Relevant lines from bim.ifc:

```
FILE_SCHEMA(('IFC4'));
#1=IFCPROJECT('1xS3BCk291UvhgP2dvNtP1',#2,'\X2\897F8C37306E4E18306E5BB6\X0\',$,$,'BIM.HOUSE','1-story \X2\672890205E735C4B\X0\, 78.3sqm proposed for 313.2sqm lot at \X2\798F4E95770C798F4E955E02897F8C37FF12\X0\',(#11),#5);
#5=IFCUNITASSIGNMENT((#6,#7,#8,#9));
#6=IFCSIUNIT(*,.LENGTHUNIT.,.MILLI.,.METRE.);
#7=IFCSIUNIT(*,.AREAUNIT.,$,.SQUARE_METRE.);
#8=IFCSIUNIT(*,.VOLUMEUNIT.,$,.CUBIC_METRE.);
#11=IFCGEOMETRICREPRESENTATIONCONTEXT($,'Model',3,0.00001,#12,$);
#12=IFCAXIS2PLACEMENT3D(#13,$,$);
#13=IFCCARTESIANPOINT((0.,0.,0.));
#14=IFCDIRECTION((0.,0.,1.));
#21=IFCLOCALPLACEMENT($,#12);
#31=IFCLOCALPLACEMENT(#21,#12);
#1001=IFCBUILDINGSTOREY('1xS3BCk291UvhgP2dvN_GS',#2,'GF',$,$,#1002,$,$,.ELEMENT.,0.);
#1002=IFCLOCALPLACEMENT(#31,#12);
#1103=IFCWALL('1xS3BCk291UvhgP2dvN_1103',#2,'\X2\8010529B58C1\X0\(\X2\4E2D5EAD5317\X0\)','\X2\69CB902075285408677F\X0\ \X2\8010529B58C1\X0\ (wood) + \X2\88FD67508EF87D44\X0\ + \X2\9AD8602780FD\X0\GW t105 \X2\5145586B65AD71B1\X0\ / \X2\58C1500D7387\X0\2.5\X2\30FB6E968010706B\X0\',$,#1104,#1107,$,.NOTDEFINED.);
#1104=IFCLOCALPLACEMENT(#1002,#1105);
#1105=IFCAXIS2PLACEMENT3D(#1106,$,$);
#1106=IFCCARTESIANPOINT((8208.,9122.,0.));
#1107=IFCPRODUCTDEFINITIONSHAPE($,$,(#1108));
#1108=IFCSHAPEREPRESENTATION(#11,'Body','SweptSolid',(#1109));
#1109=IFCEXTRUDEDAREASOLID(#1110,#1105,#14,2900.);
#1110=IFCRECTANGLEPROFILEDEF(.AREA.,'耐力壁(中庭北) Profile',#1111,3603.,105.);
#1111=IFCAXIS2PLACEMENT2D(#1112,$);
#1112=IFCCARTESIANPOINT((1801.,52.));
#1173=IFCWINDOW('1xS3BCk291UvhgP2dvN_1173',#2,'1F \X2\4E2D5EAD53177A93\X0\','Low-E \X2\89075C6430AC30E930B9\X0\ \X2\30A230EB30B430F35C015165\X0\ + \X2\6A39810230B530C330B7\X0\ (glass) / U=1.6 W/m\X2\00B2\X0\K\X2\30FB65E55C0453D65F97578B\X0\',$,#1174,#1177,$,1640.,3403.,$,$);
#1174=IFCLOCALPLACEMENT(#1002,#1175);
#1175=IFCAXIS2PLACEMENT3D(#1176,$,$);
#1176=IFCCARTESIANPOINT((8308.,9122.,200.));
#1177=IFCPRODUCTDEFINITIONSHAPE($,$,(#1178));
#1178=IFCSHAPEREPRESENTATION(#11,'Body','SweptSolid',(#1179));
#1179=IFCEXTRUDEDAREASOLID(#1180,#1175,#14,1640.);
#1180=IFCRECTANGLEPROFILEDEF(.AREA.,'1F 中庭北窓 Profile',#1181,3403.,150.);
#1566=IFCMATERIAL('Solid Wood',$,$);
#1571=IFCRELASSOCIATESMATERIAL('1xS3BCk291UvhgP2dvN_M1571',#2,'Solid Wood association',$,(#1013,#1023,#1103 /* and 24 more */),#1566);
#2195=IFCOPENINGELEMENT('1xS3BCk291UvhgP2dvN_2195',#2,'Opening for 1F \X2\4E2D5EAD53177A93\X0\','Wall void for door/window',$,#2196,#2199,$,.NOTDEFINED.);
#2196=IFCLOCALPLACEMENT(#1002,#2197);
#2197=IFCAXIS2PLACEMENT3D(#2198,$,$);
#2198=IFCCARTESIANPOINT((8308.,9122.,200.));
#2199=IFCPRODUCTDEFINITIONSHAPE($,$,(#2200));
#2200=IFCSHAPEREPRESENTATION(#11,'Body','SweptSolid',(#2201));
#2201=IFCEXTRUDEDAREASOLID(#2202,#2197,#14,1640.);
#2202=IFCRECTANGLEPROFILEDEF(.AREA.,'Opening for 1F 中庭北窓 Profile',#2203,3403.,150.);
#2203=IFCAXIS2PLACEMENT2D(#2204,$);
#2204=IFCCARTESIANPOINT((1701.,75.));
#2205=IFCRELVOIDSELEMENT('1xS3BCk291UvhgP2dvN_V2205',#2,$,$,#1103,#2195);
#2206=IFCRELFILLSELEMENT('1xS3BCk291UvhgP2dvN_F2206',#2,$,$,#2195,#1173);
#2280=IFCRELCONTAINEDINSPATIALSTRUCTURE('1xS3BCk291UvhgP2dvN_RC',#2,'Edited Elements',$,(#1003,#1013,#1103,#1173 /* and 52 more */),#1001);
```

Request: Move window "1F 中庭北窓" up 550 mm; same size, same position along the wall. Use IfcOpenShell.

```python
import numpy as np
import ifcopenshell
import ifcopenshell.api.geometry
import ifcopenshell.util.placement
import ifcopenshell.util.unit

model = ifcopenshell.open("bim.ifc")
unit_scale = ifcopenshell.util.unit.calculate_unit_scale(model)

window = model.by_guid("1xS3BCk291UvhgP2dvN_1173")
opening = window.FillsVoids[0].RelatingOpeningElement
dz = 0.55 / unit_scale

shift = np.array([0.0, 0.0, dz])
# The window is not placed relative to its opening, so move both.
for product in (opening, window):
    matrix = ifcopenshell.util.placement.get_local_placement(product.ObjectPlacement)
    matrix[:3, 3] += shift
    ifcopenshell.api.geometry.edit_object_placement(model, product=product, matrix=matrix, is_si=False)

print(f"moved by {dz * unit_scale:+.3f} m")

model.write("bim_updated.ifc")
```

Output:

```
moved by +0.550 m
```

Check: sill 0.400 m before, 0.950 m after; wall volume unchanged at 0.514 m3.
